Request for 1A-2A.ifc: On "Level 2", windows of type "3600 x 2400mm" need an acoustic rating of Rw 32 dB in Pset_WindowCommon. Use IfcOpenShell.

First a look at what the model holds.

```python
import ifcopenshell
import ifcopenshell.util.element

model = ifcopenshell.open("1A-2A.ifc")
print(model.schema)
storey = next(s for s in model.by_type("IfcBuildingStorey") if s.Name == "Level 2")
windows = [e for e in ifcopenshell.util.element.get_decomposition(storey) if e.is_a("IfcWindow")]
seen = {}
for e in windows:
    element_type = ifcopenshell.util.element.get_type(e)
    key = (element_type.Name if element_type != e and element_type else None, ifcopenshell.util.element.get_pset(e, "Pset_WindowCommon", "AcousticRating"))
    seen[key] = seen.get(key, 0) + 1
for (name, value), count in sorted(seen.items(), key=str):
    print(count, "x", name, "|", value)
```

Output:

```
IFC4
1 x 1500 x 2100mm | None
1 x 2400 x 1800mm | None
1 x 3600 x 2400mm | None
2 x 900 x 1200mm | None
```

```python
import ifcopenshell
import ifcopenshell.api.pset
import ifcopenshell.util.element

model = ifcopenshell.open("1A-2A.ifc")

storey = next(s for s in model.by_type("IfcBuildingStorey") if s.Name == "Level 2")
windows = [e for e in ifcopenshell.util.element.get_decomposition(storey) if e.is_a("IfcWindow")]

count = 0
for e in windows:
    element_type = ifcopenshell.util.element.get_type(e)
    if element_type in (None, e) or element_type.Name != "3600 x 2400mm":
        continue
    # add_pset returns the element's existing set when there is one.
    pset = ifcopenshell.api.pset.add_pset(model, product=e, name="Pset_WindowCommon")
    ifcopenshell.api.pset.edit_pset(model, pset=pset, properties={"AcousticRating": "Rw 32 dB"})
    count += 1

print(count, "windows updated")

model.write("1A-2A_updated.ifc")
```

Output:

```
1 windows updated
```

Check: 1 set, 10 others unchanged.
